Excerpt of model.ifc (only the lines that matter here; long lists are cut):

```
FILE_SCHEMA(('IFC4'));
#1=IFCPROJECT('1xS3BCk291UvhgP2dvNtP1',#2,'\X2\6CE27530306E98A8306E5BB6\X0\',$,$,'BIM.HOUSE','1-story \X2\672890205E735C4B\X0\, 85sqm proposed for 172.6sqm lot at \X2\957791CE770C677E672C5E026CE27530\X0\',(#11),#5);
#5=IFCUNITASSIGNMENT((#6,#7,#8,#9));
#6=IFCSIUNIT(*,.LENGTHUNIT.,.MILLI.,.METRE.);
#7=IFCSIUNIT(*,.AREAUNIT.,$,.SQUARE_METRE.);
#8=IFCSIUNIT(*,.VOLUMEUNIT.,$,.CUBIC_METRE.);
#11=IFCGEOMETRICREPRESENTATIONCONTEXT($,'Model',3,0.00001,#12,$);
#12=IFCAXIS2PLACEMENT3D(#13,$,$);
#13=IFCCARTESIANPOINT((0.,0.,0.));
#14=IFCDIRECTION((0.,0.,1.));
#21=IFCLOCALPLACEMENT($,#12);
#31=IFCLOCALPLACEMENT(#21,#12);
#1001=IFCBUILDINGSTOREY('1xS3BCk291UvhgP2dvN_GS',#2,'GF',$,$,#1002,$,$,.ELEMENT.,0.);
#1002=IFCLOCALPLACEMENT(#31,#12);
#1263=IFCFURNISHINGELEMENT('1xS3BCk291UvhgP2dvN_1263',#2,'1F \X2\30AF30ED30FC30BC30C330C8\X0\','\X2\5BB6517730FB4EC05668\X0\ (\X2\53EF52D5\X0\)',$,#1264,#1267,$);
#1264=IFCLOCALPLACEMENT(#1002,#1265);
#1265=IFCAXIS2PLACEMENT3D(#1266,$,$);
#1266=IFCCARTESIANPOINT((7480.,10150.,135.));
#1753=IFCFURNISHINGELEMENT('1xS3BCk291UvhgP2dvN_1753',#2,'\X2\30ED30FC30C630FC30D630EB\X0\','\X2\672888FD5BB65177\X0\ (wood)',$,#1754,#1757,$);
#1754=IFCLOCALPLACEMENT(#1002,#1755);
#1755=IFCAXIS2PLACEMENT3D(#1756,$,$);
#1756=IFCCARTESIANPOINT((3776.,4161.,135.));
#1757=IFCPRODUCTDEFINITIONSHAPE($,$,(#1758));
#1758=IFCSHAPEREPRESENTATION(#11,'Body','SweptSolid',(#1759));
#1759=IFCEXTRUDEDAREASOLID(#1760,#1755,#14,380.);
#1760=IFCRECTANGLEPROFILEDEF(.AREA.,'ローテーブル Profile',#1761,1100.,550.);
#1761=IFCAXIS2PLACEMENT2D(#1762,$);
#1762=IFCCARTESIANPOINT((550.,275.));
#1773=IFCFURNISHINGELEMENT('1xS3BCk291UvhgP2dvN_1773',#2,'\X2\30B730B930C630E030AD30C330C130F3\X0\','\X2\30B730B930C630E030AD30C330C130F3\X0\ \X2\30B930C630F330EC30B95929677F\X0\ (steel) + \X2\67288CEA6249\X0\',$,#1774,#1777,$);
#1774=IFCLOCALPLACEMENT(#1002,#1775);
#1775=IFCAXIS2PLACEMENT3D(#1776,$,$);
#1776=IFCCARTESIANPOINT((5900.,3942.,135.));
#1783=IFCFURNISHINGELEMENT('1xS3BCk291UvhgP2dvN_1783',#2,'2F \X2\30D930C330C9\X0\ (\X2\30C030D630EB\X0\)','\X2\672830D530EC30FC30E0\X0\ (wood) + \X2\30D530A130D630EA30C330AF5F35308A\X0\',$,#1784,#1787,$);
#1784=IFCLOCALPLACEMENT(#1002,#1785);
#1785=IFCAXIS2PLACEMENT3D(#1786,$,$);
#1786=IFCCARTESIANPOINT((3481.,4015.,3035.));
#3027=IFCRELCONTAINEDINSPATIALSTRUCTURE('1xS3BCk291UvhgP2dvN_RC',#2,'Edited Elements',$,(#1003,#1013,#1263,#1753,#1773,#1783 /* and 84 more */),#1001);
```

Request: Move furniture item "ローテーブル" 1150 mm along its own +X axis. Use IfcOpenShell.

```python
import ifcopenshell
import ifcopenshell.api.geometry
import ifcopenshell.util.placement
import ifcopenshell.util.unit

model = ifcopenshell.open("model.ifc")
unit_scale = ifcopenshell.util.unit.calculate_unit_scale(model)

item = model.by_guid("1xS3BCk291UvhgP2dvN_1753")
matrix = ifcopenshell.util.placement.get_local_placement(item.ObjectPlacement)
matrix[:3, 3] += matrix[:3, 0] * 1.15 / unit_scale
ifcopenshell.api.geometry.edit_object_placement(model, product=item, matrix=matrix, is_si=False)

print(ifcopenshell.util.placement.get_local_placement(item.ObjectPlacement).round(3) + 0.0)

model.write("model_v2.ifc")
```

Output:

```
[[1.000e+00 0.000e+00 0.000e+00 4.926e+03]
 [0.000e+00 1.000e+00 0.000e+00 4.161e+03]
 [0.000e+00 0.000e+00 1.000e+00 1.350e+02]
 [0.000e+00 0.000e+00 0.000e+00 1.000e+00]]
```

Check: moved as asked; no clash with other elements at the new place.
